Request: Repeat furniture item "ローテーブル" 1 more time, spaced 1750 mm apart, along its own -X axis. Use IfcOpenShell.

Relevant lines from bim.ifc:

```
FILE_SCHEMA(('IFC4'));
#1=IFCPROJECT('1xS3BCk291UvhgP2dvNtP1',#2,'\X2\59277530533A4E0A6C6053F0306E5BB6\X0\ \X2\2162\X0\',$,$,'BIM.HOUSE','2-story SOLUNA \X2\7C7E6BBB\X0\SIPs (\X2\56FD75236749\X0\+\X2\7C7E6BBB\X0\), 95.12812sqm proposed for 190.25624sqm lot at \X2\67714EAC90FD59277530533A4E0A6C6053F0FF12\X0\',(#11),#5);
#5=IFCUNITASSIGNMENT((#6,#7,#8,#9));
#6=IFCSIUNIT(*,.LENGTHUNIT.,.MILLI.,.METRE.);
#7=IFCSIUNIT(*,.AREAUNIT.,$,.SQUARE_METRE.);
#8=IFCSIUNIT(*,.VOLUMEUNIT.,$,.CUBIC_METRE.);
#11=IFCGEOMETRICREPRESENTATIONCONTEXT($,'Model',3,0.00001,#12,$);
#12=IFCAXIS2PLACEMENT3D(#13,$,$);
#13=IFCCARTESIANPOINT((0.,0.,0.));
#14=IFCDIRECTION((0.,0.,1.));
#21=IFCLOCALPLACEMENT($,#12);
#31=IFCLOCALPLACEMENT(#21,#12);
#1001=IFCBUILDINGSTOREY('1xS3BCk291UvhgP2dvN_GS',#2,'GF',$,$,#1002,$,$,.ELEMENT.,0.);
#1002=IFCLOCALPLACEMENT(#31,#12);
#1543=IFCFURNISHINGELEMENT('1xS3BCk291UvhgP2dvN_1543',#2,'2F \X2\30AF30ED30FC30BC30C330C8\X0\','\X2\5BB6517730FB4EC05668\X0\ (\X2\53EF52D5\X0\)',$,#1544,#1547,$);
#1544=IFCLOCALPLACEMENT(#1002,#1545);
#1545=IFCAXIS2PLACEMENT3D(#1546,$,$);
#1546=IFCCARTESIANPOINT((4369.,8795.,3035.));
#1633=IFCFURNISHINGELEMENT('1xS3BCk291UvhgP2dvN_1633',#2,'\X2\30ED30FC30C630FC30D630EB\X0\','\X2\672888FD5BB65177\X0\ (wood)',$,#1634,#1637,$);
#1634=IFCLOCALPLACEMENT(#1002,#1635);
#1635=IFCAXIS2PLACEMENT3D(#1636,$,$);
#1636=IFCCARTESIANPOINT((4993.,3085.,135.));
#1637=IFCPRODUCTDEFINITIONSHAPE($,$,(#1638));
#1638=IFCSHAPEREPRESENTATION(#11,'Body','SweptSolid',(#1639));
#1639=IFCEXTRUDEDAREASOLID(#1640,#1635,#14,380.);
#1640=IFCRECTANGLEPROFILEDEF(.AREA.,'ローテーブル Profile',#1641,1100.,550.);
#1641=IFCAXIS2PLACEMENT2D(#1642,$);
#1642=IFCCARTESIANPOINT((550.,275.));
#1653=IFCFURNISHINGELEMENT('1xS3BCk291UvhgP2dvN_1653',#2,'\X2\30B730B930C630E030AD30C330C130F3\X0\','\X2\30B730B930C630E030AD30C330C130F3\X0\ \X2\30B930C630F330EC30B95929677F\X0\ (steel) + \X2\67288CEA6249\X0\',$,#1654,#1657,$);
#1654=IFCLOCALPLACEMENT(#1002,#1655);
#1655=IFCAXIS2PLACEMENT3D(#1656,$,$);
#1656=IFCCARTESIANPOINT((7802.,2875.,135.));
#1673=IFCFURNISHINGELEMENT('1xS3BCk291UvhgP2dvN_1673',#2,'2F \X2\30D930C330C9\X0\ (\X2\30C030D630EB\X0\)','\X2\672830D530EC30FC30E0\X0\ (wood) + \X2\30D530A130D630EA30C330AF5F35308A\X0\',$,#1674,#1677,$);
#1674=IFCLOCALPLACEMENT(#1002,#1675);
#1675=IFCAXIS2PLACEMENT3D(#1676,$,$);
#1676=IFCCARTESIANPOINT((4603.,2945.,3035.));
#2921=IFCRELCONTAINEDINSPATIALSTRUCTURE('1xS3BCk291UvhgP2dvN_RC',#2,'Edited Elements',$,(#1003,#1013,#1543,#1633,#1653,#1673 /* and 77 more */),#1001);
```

```python
import ifcopenshell
import ifcopenshell.api.geometry
import ifcopenshell.api.root
import ifcopenshell.util.element
import ifcopenshell.util.placement

model = ifcopenshell.open("bim.ifc")


def reuse_history(source, copy):
    """copy_class also copies each property set's owner history, people and application; keep the originals."""
    for rel in copy.IsDefinedBy:
        if rel.is_a("IfcRelDefinesByProperties") and (history := rel.RelatingPropertyDefinition.OwnerHistory):
            rel.RelatingPropertyDefinition.OwnerHistory = source.OwnerHistory
            ifcopenshell.util.element.remove_deep2(model, history)


source = model.by_guid("1xS3BCk291UvhgP2dvN_1633")
base = ifcopenshell.util.placement.get_local_placement(source.ObjectPlacement)
step = -base[:3, 0] * 1750.0

for i in range(1, 2):
    copy = ifcopenshell.api.root.copy_class(model, product=source)
    copy.Representation = ifcopenshell.util.element.copy_deep(
        model, source.Representation, exclude=["IfcGeometricRepresentationContext", "IfcRepresentationMap"]
    )
    reuse_history(source, copy)
    matrix = base.copy()
    matrix[:3, 3] += i * step
    print("added at", matrix[:3, 3].round(3) + 0.0)
    ifcopenshell.api.geometry.edit_object_placement(model, product=copy, matrix=matrix, is_si=False)

model.write("bim_v2.ifc")
```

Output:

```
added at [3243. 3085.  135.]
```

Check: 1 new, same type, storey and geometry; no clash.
